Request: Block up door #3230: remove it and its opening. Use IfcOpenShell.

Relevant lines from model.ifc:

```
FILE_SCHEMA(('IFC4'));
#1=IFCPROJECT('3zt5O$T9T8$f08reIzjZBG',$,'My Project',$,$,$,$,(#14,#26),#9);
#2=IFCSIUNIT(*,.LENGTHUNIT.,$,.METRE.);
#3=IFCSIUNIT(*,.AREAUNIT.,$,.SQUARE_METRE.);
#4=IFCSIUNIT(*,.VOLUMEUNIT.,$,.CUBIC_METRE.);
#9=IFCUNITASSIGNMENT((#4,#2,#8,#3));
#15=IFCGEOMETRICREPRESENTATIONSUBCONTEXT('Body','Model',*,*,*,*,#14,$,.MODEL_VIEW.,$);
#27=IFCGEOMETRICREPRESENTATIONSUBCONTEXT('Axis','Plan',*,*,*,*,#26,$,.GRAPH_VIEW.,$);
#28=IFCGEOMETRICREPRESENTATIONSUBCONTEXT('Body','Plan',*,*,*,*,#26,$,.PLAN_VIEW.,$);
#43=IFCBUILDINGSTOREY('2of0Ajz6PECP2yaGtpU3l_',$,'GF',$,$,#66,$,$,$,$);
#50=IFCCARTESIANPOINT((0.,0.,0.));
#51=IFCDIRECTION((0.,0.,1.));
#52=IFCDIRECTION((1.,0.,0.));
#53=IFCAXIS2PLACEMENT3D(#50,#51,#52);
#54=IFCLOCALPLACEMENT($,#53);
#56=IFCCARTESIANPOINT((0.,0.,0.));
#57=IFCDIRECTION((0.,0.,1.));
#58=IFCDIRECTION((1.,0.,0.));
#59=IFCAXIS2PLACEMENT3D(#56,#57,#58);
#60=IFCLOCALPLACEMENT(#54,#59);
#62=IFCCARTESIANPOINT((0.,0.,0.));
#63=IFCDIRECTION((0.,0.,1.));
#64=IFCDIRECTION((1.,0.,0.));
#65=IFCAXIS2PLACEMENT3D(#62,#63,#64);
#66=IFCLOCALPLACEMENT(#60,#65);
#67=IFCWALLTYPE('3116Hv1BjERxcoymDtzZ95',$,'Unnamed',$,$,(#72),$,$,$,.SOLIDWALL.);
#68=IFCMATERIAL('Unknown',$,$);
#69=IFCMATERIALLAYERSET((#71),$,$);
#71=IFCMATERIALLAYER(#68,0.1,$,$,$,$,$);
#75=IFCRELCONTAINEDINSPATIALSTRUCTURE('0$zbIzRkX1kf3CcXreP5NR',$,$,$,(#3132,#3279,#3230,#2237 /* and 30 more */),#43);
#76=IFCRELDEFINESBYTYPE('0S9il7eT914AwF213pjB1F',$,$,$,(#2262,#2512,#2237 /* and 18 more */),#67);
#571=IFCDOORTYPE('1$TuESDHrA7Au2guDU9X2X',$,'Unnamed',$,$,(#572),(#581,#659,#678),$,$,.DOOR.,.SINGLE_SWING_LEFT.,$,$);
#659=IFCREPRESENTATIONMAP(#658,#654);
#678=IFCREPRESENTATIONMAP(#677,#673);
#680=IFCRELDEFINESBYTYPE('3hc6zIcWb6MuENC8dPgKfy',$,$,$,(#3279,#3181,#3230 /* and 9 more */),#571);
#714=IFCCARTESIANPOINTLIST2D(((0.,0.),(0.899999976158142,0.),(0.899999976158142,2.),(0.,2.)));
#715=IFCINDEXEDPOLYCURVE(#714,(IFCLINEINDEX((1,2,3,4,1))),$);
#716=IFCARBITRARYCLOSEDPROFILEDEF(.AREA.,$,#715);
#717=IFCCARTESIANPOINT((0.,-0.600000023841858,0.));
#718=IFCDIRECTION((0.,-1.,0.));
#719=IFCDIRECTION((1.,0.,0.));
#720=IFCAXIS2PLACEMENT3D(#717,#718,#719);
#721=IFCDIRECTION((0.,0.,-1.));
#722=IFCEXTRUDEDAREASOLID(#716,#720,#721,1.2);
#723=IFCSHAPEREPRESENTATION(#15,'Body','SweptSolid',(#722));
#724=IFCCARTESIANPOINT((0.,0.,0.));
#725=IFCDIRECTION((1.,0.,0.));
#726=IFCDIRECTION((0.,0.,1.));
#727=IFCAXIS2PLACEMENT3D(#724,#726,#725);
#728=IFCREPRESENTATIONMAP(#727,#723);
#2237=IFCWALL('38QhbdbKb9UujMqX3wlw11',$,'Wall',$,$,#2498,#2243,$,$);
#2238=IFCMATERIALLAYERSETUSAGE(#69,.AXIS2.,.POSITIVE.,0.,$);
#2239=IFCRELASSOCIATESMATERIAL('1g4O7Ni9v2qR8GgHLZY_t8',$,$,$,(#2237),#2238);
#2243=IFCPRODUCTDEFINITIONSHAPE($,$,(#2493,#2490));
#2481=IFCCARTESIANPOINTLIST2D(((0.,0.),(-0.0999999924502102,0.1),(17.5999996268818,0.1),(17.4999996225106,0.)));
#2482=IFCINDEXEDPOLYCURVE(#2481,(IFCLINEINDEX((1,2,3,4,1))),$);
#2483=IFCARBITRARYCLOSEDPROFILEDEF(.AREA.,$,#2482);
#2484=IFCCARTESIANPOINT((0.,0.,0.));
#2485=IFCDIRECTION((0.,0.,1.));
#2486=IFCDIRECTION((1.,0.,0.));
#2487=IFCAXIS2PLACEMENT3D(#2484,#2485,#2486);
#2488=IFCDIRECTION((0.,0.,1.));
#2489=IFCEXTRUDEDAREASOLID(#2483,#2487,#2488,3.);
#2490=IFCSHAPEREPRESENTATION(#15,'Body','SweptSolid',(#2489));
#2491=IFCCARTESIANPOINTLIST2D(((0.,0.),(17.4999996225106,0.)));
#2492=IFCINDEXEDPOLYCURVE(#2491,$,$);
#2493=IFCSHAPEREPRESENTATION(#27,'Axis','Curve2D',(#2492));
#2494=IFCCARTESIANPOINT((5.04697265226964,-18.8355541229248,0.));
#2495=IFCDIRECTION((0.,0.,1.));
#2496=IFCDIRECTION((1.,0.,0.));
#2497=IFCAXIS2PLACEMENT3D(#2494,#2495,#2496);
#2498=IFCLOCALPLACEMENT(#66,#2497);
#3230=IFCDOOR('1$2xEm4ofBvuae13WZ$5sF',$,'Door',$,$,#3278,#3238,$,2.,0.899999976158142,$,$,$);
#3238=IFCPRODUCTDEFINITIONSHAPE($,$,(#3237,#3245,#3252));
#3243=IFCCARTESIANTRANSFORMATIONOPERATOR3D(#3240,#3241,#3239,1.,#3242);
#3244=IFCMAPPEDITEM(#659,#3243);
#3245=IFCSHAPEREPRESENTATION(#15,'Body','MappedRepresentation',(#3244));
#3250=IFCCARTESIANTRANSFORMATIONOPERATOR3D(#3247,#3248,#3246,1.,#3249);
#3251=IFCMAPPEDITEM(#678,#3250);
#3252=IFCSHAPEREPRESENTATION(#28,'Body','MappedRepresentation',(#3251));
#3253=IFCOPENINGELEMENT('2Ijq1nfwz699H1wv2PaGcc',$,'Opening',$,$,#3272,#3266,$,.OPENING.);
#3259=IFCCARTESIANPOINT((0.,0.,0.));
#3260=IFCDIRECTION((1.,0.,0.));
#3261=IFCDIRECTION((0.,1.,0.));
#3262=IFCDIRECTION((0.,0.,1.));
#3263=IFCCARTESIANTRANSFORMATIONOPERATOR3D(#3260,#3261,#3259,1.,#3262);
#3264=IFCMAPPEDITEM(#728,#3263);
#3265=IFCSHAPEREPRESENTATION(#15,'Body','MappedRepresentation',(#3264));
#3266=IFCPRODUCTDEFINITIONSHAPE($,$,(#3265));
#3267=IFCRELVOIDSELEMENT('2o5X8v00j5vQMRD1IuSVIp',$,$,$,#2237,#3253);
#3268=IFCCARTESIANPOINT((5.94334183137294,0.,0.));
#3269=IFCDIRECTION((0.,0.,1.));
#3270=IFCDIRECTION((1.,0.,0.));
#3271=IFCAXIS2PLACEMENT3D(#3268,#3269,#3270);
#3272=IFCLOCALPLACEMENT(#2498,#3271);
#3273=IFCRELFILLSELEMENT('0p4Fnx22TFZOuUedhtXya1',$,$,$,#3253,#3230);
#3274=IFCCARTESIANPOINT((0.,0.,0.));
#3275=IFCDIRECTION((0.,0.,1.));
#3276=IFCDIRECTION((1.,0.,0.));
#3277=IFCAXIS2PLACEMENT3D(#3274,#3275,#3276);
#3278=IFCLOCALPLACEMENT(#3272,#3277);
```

```python
import ifcopenshell
import ifcopenshell.api.feature
import ifcopenshell.api.root
import ifcopenshell.geom
import ifcopenshell.util.shape

model = ifcopenshell.open("model.ifc")
settings = ifcopenshell.geom.settings()


def volume(element):
    """Net volume in cubic metres, openings subtracted."""
    shape = ifcopenshell.geom.create_shape(settings, element)
    return ifcopenshell.util.shape.get_volume(shape.geometry)


door = model.by_guid("1$2xEm4ofBvuae13WZ$5sF")
opening = door.FillsVoids[0].RelatingOpeningElement
wall = opening.VoidsElements[0].RelatingBuildingElement
before = volume(wall)

ifcopenshell.api.root.remove_product(model, product=door)
ifcopenshell.api.feature.remove_feature(model, feature=opening)

after = volume(wall)

print(f"wall volume {before:.3f} -> {after:.3f} m3")

model.write("model-out.ifc")
```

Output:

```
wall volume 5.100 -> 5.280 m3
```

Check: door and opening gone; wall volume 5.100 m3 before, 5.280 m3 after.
